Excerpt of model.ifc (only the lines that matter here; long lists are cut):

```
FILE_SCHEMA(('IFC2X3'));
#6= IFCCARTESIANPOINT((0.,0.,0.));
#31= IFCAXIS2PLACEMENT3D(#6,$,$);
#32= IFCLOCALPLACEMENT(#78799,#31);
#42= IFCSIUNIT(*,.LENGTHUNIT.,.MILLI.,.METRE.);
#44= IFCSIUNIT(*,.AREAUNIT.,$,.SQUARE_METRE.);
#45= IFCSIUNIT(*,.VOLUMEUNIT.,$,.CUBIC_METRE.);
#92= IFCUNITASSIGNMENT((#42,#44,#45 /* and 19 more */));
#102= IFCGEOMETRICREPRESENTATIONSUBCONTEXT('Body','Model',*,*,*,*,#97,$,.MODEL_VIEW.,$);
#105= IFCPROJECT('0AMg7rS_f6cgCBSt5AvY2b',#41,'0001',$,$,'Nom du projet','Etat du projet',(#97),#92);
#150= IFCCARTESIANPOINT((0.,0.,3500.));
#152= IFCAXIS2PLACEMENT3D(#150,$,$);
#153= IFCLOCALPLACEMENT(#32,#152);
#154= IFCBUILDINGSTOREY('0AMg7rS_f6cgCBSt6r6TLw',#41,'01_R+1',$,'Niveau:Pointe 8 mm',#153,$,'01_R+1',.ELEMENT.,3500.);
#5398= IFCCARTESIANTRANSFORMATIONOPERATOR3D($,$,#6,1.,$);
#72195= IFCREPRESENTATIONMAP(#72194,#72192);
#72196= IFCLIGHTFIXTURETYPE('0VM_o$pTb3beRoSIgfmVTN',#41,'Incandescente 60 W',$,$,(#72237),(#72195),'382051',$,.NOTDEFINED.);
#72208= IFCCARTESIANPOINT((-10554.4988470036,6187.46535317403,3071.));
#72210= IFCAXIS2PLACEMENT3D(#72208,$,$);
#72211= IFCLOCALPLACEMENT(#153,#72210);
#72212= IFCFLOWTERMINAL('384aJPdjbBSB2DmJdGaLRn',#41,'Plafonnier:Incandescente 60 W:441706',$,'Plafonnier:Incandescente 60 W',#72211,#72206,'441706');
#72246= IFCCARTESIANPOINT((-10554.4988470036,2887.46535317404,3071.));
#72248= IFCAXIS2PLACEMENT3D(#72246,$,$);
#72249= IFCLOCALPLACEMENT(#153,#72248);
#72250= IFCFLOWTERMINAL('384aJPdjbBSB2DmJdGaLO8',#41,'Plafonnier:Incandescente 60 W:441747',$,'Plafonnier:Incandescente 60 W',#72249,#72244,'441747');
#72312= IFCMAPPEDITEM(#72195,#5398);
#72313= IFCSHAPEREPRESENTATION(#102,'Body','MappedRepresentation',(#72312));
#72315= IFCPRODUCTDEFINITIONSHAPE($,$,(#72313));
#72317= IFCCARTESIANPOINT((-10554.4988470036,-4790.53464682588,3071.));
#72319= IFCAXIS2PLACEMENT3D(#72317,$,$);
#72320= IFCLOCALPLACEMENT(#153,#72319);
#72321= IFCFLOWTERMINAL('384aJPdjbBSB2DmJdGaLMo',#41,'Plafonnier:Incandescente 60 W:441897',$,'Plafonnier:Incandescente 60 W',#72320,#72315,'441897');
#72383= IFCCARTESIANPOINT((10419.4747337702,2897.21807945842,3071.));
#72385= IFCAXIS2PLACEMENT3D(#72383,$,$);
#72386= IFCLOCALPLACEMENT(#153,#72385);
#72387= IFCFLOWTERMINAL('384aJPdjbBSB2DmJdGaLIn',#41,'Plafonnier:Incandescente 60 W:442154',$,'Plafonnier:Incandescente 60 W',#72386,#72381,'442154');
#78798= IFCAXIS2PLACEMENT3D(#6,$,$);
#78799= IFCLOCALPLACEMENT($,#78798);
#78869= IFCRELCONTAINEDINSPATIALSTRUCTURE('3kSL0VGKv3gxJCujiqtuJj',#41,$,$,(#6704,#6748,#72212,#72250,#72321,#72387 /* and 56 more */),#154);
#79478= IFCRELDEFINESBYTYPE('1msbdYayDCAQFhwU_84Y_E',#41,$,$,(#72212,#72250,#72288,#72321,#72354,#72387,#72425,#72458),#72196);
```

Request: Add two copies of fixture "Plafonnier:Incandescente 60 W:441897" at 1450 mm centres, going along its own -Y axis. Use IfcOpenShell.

```python
import ifcopenshell
import ifcopenshell.api.geometry
import ifcopenshell.api.root
import ifcopenshell.util.element
import ifcopenshell.util.placement
import ifcopenshell.util.unit

model = ifcopenshell.open("model.ifc")
unit_scale = ifcopenshell.util.unit.calculate_unit_scale(model)


def reuse_history(source, copy):
    """copy_class also copies each property set's owner history, people and application; keep the originals."""
    for rel in copy.IsDefinedBy:
        if rel.is_a("IfcRelDefinesByProperties") and (history := rel.RelatingPropertyDefinition.OwnerHistory):
            rel.RelatingPropertyDefinition.OwnerHistory = source.OwnerHistory
            ifcopenshell.util.element.remove_deep2(model, history)


source = model.by_guid("384aJPdjbBSB2DmJdGaLMo")
base = ifcopenshell.util.placement.get_local_placement(source.ObjectPlacement)
step = -base[:3, 1] * 1.45 / unit_scale

for i in range(1, 3):
    copy = ifcopenshell.api.root.copy_class(model, product=source)
    copy.Representation = ifcopenshell.util.element.copy_deep(
        model, source.Representation, exclude=["IfcGeometricRepresentationContext", "IfcRepresentationMap"]
    )
    copy.Name = "Plafonnier:Incandescente 60 W"
    copy.Tag = None
    reuse_history(source, copy)
    matrix = base.copy()
    matrix[:3, 3] += i * step
    print("added at", matrix[:3, 3].round(3) + 0.0)
    ifcopenshell.api.geometry.edit_object_placement(model, product=copy, matrix=matrix, is_si=False)

model.write("model_updated.ifc")
```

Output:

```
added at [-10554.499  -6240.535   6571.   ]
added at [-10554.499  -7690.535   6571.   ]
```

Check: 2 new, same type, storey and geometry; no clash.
